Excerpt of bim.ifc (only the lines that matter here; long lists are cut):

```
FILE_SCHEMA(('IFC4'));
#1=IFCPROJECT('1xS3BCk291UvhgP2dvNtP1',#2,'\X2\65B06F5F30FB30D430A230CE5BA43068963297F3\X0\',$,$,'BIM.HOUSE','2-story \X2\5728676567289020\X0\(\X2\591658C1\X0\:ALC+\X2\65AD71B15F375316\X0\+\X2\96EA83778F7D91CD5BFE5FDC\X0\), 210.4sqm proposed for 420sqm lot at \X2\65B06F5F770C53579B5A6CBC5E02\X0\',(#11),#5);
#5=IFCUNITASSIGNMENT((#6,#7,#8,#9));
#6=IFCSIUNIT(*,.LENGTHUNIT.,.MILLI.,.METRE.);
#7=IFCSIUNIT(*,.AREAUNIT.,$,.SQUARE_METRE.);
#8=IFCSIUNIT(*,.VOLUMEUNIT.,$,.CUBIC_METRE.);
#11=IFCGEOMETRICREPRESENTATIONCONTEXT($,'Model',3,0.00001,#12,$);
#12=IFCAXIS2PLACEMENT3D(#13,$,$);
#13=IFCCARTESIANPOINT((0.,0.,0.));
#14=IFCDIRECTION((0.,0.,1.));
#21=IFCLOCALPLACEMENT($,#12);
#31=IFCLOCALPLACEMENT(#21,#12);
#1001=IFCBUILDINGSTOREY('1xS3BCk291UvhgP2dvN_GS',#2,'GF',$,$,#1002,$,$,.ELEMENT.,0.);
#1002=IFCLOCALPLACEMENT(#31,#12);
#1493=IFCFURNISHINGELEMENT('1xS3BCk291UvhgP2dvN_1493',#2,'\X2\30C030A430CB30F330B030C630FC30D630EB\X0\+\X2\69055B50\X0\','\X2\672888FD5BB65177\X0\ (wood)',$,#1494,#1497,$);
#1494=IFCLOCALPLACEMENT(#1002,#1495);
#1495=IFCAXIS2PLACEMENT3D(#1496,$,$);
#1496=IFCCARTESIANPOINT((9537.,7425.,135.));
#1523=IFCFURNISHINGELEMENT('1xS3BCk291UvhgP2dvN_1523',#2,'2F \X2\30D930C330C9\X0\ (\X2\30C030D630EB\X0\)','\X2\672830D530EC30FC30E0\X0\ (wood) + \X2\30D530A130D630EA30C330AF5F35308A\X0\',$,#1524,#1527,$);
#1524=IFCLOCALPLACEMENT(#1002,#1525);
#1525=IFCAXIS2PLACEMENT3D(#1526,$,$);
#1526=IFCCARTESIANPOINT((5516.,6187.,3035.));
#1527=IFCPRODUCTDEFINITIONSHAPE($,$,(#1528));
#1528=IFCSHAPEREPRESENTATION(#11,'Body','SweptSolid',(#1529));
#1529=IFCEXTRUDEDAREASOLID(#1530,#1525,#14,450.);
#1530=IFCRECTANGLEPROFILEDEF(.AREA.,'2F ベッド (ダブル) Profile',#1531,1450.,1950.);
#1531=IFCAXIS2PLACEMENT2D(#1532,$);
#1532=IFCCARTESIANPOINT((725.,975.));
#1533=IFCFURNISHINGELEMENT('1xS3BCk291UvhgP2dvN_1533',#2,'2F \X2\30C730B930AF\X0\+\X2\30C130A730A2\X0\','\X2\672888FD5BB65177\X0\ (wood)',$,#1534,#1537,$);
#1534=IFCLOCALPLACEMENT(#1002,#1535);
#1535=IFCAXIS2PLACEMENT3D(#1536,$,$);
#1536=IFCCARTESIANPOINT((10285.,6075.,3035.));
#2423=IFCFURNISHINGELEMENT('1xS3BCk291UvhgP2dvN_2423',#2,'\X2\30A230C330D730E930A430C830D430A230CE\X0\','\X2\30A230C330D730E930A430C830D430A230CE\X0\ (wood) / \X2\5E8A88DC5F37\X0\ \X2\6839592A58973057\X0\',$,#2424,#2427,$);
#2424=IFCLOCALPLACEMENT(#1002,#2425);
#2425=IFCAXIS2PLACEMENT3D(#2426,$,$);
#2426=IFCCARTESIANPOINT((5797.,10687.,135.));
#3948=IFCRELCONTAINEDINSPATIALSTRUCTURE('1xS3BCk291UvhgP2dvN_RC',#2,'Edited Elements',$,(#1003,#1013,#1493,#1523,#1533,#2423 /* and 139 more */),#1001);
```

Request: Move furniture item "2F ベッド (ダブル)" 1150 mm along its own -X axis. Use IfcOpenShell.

```python
import ifcopenshell
import ifcopenshell.api.geometry
import ifcopenshell.util.placement

model = ifcopenshell.open("bim.ifc")

item = model.by_guid("1xS3BCk291UvhgP2dvN_1523")
matrix = ifcopenshell.util.placement.get_local_placement(item.ObjectPlacement)
matrix[:3, 3] -= matrix[:3, 0] * 1150.0
ifcopenshell.api.geometry.edit_object_placement(model, product=item, matrix=matrix, is_si=False)

print(ifcopenshell.util.placement.get_local_placement(item.ObjectPlacement).round(3) + 0.0)

model.write("bim_edited.ifc")
```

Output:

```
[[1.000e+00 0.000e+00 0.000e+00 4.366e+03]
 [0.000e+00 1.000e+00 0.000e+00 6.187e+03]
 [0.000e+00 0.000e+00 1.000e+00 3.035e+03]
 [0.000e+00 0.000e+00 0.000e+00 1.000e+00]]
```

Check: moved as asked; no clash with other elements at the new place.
